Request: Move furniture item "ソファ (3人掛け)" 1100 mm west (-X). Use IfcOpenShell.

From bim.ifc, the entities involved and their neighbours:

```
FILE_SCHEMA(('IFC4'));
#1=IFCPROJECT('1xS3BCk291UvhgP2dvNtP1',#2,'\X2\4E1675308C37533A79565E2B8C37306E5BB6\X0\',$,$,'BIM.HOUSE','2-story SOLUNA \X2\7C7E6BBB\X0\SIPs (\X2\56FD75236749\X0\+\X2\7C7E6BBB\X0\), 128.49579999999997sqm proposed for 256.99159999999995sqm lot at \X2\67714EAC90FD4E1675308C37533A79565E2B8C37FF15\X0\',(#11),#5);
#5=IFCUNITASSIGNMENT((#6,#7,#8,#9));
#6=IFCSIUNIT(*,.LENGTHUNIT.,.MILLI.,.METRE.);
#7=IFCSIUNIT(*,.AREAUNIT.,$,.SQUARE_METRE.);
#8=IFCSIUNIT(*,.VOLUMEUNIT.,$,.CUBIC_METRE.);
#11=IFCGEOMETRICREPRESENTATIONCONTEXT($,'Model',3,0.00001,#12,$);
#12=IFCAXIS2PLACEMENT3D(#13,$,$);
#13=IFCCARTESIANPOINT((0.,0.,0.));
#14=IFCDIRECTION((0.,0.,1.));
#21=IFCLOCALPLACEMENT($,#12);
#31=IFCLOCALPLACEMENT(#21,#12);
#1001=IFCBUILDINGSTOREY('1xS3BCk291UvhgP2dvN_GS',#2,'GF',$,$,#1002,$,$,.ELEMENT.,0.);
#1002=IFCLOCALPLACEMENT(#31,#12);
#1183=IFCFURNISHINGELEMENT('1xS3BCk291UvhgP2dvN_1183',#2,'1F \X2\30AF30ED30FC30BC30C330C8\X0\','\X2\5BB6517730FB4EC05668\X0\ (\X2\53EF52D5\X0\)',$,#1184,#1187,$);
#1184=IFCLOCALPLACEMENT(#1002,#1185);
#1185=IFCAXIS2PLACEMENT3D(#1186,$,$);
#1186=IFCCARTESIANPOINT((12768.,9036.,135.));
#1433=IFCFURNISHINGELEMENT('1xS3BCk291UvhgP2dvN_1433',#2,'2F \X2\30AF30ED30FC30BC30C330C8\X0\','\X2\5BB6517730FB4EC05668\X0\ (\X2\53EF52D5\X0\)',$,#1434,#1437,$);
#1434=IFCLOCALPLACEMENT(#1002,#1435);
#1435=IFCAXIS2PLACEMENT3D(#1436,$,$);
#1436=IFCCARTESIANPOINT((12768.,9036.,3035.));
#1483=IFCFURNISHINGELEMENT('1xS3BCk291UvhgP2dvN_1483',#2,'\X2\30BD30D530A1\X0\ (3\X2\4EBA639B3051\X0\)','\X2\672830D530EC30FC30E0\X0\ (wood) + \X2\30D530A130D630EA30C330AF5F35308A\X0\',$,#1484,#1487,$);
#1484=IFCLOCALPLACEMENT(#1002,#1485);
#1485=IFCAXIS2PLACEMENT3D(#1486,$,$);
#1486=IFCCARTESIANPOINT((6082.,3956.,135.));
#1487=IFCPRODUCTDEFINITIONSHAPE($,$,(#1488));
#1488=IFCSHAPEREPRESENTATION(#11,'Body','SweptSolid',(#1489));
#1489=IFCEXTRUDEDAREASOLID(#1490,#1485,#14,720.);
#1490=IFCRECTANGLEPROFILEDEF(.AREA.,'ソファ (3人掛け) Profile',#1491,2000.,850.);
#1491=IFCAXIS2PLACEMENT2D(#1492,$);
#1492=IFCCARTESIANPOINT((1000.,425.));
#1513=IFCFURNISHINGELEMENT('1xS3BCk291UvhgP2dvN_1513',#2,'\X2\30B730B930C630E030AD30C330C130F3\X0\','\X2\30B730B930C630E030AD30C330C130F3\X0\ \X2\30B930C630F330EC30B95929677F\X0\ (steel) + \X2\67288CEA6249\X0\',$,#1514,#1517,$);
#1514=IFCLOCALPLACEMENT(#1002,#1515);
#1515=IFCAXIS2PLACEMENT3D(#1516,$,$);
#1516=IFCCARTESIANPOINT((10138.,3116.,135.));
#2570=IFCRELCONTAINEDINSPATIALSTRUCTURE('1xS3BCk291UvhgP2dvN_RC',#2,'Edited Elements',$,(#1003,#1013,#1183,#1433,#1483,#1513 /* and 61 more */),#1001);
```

```python
import ifcopenshell
import ifcopenshell.api.geometry
import ifcopenshell.util.placement
import ifcopenshell.util.unit

model = ifcopenshell.open("bim.ifc")
unit_scale = ifcopenshell.util.unit.calculate_unit_scale(model)

item = model.by_guid("1xS3BCk291UvhgP2dvN_1483")
matrix = ifcopenshell.util.placement.get_local_placement(item.ObjectPlacement)
matrix[0, 3] -= 1.1 / unit_scale
ifcopenshell.api.geometry.edit_object_placement(model, product=item, matrix=matrix, is_si=False)

print(ifcopenshell.util.placement.get_local_placement(item.ObjectPlacement).round(3) + 0.0)

model.write("bim_rev.ifc")
```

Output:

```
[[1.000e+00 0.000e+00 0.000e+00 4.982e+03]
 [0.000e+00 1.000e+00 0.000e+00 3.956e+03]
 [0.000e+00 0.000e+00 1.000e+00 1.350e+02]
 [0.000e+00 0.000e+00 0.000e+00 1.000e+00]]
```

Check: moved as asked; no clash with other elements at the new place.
